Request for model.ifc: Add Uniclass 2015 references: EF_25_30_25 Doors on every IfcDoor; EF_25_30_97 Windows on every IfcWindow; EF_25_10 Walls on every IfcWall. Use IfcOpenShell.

First a look at what the model holds.

```python
import ifcopenshell

model = ifcopenshell.open("model.ifc")
print(model.schema)
print("classifications:", [c.Name for c in model.by_type("IfcClassification")])
for ifc_class in ("IfcDoor", "IfcRoof", "IfcStair", "IfcWall", "IfcWindow"):
    print(ifc_class, len(model.by_type(ifc_class)))
```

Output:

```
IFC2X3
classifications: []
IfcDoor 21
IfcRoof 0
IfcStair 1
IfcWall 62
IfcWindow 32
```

```python
import ifcopenshell
import ifcopenshell.api.classification

model = ifcopenshell.open("model.ifc")

# IFC2X3 requires Source and Edition and has no link from the project to the system.
system = model.create_entity("IfcClassification", Source="NBS", Edition="2015", Name="Uniclass 2015")

codes = {
    "IfcDoor": ("EF_25_30_25", "Doors"),
    "IfcWindow": ("EF_25_30_97", "Windows"),
    "IfcWall": ("EF_25_10", "Walls"),
}
for ifc_class, (code, name) in codes.items():
    products = model.by_type(ifc_class)
    ifcopenshell.api.classification.add_reference(
        model, products=products, classification=system, identification=code, name=name
    )
    print(code, len(products))

model.write("model_edited.ifc")
```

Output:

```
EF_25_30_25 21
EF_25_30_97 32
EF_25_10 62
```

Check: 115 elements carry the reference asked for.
